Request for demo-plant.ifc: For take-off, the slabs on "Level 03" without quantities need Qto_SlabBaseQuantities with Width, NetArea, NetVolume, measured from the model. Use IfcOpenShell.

First a look at what the model holds.

```python
import ifcopenshell
import ifcopenshell.util.element
import ifcopenshell.util.unit

model = ifcopenshell.open("demo-plant.ifc")
print(model.schema)
for unit_type in ("LENGTHUNIT", "AREAUNIT", "VOLUMEUNIT"):
    print(unit_type, ifcopenshell.util.unit.calculate_unit_scale(model, unit_type))
storey = next(s for s in model.by_type("IfcBuildingStorey") if s.Name == "Level 03")
slabs = [e for e in ifcopenshell.util.element.get_decomposition(storey) if e.is_a("IfcSlab")]
for e in sorted(slabs, key=lambda e: e.id()):
    print(e.id(), e.is_a(), e.Name, list(ifcopenshell.util.element.get_psets(e, qtos_only=True)), sep=" | ")
```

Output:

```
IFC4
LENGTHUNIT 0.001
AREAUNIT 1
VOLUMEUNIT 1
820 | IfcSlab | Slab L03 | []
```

```python
import ifcopenshell
import ifcopenshell.api.pset
import ifcopenshell.geom
import ifcopenshell.util.element
import ifcopenshell.util.shape
import ifcopenshell.util.unit

model = ifcopenshell.open("demo-plant.ifc")
unit_scale = ifcopenshell.util.unit.calculate_unit_scale(model)
area_scale = ifcopenshell.util.unit.calculate_unit_scale(model, "AREAUNIT")
volume_scale = ifcopenshell.util.unit.calculate_unit_scale(model, "VOLUMEUNIT")
settings = ifcopenshell.geom.settings()

storey = next(s for s in model.by_type("IfcBuildingStorey") if s.Name == "Level 03")
slabs = [e for e in ifcopenshell.util.element.get_decomposition(storey) if e.is_a("IfcSlab")]

for e in sorted(slabs, key=lambda e: e.id()):
    if ifcopenshell.util.element.get_psets(e, qtos_only=True, should_inherit=False):
        continue
    # Geometry comes back in metres, in the element's own axes.
    shape = ifcopenshell.geom.create_shape(settings, e)
    values = {
        "Width": ifcopenshell.util.shape.get_z(shape.geometry) / unit_scale,
        "NetArea": ifcopenshell.util.shape.get_footprint_area(shape.geometry) / area_scale,
        "NetVolume": ifcopenshell.util.shape.get_volume(shape.geometry) / volume_scale,
    }
    qto = ifcopenshell.api.pset.add_qto(model, product=e, name="Qto_SlabBaseQuantities")
    ifcopenshell.api.pset.edit_qto(model, qto=qto, properties=values)
    print(e.id(), {k: round(v, 3) for k, v in values.items()})

model.write("demo-plant_updated.ifc")
```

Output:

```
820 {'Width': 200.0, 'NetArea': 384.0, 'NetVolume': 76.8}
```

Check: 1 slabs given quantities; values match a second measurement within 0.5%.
